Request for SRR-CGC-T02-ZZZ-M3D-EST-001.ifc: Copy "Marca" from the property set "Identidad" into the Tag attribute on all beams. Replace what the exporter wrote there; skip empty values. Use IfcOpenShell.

First a look at what the model holds.

```python
import ifcopenshell
import ifcopenshell.util.element

model = ifcopenshell.open("SRR-CGC-T02-ZZZ-M3D-EST-001.ifc")
print(model.schema)
beams = model.by_type("IfcBeam")
print(len(beams), "beams")
for e in beams[:8]:
    source = ifcopenshell.util.element.get_pset(e, "Identidad", "Marca")
    target = e.Tag
    print(e.id(), repr(source), repr(target), sep=" | ")
```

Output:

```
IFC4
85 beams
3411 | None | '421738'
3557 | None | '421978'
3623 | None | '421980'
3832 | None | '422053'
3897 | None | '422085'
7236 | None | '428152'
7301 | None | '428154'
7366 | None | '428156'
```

```python
import ifcopenshell
import ifcopenshell.util.element

model = ifcopenshell.open("SRR-CGC-T02-ZZZ-M3D-EST-001.ifc")

count = 0
for e in model.by_type("IfcBeam"):
    value = ifcopenshell.util.element.get_pset(e, "Identidad", "Marca")
    current = e.Tag
    if not value or not value.strip() or current == value:
        continue
    e.Tag = value
    count += 1

print(count, "beams updated")

model.write("SRR-CGC-T02-ZZZ-M3D-EST-001_edited.ifc")
```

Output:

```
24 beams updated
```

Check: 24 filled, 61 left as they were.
